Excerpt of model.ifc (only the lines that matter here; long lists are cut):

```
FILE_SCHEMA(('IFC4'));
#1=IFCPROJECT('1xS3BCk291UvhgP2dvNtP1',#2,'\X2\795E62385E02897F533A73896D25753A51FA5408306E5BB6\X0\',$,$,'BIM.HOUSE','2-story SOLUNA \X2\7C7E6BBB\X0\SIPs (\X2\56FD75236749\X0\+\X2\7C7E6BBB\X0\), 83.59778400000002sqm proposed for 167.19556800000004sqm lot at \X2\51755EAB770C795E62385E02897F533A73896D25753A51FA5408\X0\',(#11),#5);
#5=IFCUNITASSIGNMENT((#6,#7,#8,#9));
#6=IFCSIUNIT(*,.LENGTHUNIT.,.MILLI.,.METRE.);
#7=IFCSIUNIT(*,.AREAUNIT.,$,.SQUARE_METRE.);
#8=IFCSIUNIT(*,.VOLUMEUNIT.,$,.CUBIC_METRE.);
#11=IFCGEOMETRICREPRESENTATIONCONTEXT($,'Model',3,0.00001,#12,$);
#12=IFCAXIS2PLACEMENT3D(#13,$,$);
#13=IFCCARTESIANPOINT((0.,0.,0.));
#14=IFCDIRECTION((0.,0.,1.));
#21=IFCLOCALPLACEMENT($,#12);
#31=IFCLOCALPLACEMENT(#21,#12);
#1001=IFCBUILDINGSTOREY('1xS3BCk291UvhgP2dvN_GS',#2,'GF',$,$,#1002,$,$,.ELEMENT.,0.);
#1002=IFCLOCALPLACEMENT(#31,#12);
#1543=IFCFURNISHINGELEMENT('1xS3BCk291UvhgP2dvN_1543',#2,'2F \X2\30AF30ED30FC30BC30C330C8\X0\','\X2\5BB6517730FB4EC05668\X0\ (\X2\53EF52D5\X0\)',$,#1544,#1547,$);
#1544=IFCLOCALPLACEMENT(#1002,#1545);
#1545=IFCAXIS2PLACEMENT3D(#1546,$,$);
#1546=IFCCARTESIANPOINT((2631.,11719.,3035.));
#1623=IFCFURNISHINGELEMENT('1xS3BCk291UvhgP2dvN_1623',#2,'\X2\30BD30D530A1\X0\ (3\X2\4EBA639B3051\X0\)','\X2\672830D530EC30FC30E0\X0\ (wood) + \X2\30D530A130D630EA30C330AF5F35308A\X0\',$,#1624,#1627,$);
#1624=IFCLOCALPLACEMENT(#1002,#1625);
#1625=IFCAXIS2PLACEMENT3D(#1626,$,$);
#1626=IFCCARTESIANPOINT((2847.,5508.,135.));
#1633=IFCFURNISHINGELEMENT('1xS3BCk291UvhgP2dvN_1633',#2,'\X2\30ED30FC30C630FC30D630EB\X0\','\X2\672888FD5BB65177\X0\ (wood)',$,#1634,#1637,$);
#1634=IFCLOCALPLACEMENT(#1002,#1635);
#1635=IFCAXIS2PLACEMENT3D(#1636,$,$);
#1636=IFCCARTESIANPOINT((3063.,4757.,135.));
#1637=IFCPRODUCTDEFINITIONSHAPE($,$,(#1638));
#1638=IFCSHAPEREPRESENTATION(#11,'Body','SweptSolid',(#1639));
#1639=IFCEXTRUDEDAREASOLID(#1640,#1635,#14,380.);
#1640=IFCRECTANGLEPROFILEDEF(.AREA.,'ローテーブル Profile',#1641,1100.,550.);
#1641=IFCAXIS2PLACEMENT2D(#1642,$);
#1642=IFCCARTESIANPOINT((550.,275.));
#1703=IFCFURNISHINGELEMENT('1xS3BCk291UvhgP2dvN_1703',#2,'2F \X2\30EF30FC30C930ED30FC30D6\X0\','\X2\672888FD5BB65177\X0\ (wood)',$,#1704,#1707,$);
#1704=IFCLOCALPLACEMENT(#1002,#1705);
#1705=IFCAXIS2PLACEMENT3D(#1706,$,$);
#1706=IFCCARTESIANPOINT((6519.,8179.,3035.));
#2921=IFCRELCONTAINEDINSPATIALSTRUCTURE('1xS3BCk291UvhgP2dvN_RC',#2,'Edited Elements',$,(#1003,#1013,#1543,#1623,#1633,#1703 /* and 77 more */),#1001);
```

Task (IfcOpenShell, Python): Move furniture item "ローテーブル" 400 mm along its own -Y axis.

```python
import ifcopenshell
import ifcopenshell.api.geometry
import ifcopenshell.util.placement

model = ifcopenshell.open("model.ifc")

item = model.by_guid("1xS3BCk291UvhgP2dvN_1633")
matrix = ifcopenshell.util.placement.get_local_placement(item.ObjectPlacement)
matrix[:3, 3] -= matrix[:3, 1] * 400.0
ifcopenshell.api.geometry.edit_object_placement(model, product=item, matrix=matrix, is_si=False)

print(ifcopenshell.util.placement.get_local_placement(item.ObjectPlacement).round(3) + 0.0)

model.write("model-out.ifc")
```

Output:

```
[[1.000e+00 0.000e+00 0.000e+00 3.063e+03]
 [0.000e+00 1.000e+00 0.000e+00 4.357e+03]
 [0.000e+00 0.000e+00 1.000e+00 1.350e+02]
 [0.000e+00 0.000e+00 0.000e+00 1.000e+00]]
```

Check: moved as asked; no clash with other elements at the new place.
